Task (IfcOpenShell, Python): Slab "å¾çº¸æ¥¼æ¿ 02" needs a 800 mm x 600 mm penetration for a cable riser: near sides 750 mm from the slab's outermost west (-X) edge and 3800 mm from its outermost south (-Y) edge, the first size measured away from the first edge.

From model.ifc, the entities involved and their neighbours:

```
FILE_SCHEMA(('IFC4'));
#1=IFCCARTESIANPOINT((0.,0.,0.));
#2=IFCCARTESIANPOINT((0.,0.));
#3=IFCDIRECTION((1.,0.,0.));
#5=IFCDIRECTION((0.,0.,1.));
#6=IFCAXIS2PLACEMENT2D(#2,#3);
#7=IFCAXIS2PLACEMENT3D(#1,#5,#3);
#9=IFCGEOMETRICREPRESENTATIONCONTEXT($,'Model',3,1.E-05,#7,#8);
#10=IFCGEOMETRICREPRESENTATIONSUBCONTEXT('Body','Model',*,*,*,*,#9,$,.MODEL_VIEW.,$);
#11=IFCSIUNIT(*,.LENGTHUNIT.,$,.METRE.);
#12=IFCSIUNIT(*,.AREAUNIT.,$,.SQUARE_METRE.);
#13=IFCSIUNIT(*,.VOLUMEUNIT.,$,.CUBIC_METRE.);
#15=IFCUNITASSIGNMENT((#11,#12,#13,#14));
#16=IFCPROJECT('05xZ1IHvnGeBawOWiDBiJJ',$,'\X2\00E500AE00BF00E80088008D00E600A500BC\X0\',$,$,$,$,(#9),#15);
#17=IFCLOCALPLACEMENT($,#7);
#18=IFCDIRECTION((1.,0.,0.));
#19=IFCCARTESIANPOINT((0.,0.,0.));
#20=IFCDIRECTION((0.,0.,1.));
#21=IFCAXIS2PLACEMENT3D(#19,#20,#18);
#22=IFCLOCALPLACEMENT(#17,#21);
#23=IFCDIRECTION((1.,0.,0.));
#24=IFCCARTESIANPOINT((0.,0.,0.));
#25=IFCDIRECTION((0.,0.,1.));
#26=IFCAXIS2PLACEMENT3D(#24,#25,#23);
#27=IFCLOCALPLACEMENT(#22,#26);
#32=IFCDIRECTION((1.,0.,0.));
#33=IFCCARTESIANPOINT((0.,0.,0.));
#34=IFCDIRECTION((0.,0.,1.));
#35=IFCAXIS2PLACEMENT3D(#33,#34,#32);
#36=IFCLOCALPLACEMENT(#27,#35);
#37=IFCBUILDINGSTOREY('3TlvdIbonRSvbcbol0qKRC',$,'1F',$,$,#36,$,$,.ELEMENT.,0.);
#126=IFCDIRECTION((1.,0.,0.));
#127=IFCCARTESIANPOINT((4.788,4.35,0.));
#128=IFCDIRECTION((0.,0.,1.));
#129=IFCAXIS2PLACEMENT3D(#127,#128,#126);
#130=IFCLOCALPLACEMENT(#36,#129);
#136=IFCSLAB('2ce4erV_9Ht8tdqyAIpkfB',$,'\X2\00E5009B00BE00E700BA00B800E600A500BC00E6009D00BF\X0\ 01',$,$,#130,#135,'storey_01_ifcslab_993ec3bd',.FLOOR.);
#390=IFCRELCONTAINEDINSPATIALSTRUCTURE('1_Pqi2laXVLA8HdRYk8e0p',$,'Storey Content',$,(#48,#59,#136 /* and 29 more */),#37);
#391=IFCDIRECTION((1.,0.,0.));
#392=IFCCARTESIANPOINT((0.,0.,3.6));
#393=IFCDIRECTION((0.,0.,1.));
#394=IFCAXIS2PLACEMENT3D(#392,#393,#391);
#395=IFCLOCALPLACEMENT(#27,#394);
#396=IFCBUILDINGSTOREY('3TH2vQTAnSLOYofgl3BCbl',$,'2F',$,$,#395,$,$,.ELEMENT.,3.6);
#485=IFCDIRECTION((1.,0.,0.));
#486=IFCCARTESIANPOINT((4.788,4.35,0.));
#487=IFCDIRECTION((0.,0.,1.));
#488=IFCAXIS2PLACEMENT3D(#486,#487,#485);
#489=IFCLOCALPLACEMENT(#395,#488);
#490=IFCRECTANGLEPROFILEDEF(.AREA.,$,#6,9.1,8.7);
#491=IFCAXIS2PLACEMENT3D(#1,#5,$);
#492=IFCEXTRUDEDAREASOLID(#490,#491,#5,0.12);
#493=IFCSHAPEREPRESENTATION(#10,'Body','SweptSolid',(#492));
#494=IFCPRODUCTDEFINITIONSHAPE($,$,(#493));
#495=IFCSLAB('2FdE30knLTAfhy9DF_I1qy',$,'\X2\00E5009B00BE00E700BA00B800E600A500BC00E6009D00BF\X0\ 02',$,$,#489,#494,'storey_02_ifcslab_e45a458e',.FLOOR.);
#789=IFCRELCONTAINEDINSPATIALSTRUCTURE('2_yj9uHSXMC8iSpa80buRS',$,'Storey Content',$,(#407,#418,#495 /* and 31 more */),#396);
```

```python
import numpy as np
import ifcopenshell
import ifcopenshell.api.feature
import ifcopenshell.api.geometry
import ifcopenshell.api.root
import ifcopenshell.geom
import ifcopenshell.util.placement
import ifcopenshell.util.representation
import ifcopenshell.util.shape
import ifcopenshell.util.unit

model = ifcopenshell.open("model.ifc")
unit_scale = ifcopenshell.util.unit.calculate_unit_scale(model)
settings = ifcopenshell.geom.settings()


def volume(element):
    """Net volume in cubic metres, openings subtracted."""
    shape = ifcopenshell.geom.create_shape(settings, element)
    return ifcopenshell.util.shape.get_volume(shape.geometry)


slab = model.by_guid("2FdE30knLTAfhy9DF_I1qy")
before = volume(slab)

# Extent in the slab's own axes, in metres. The edges named are its -X and -Y sides.
slab_shape = ifcopenshell.geom.create_shape(settings, slab)
vertices = ifcopenshell.util.shape.get_vertices(slab_shape.geometry)
x_min, y_min, bottom = vertices.min(axis=0)
top = vertices[:, 2].max()

opening = ifcopenshell.api.root.create_entity(model, ifc_class="IfcOpeningElement", name="Cable riser opening", predefined_type="OPENING")
context = ifcopenshell.util.representation.get_context(model, "Model", "Body", "MODEL_VIEW")
width, depth = 0.8, 0.6
outline = [(0.0, 0.0), (width, 0.0), (width, depth), (0.0, depth), (0.0, 0.0)]
# Overshoot both faces by 50 mm so the cut is clean.
shape = ifcopenshell.api.geometry.add_slab_representation(
    model, context=context, depth=top - bottom + 0.1, polyline=outline
)
ifcopenshell.api.geometry.assign_representation(model, product=opening, representation=shape)

matrix = ifcopenshell.util.placement.get_local_placement(slab.ObjectPlacement)
matrix[:, 3] = matrix @ np.append(np.array([x_min + 0.75, y_min + 3.8, bottom - 0.05]) / unit_scale, 1.0)
ifcopenshell.api.geometry.edit_object_placement(model, product=opening, matrix=matrix, is_si=False)
ifcopenshell.api.feature.add_feature(model, feature=opening, element=slab)

after = volume(slab)

print(f"slab volume {before:.3f} -> {after:.3f} m3")

model.write("model_edited.ifc")
```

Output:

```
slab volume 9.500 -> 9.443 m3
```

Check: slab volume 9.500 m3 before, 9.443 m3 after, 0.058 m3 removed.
